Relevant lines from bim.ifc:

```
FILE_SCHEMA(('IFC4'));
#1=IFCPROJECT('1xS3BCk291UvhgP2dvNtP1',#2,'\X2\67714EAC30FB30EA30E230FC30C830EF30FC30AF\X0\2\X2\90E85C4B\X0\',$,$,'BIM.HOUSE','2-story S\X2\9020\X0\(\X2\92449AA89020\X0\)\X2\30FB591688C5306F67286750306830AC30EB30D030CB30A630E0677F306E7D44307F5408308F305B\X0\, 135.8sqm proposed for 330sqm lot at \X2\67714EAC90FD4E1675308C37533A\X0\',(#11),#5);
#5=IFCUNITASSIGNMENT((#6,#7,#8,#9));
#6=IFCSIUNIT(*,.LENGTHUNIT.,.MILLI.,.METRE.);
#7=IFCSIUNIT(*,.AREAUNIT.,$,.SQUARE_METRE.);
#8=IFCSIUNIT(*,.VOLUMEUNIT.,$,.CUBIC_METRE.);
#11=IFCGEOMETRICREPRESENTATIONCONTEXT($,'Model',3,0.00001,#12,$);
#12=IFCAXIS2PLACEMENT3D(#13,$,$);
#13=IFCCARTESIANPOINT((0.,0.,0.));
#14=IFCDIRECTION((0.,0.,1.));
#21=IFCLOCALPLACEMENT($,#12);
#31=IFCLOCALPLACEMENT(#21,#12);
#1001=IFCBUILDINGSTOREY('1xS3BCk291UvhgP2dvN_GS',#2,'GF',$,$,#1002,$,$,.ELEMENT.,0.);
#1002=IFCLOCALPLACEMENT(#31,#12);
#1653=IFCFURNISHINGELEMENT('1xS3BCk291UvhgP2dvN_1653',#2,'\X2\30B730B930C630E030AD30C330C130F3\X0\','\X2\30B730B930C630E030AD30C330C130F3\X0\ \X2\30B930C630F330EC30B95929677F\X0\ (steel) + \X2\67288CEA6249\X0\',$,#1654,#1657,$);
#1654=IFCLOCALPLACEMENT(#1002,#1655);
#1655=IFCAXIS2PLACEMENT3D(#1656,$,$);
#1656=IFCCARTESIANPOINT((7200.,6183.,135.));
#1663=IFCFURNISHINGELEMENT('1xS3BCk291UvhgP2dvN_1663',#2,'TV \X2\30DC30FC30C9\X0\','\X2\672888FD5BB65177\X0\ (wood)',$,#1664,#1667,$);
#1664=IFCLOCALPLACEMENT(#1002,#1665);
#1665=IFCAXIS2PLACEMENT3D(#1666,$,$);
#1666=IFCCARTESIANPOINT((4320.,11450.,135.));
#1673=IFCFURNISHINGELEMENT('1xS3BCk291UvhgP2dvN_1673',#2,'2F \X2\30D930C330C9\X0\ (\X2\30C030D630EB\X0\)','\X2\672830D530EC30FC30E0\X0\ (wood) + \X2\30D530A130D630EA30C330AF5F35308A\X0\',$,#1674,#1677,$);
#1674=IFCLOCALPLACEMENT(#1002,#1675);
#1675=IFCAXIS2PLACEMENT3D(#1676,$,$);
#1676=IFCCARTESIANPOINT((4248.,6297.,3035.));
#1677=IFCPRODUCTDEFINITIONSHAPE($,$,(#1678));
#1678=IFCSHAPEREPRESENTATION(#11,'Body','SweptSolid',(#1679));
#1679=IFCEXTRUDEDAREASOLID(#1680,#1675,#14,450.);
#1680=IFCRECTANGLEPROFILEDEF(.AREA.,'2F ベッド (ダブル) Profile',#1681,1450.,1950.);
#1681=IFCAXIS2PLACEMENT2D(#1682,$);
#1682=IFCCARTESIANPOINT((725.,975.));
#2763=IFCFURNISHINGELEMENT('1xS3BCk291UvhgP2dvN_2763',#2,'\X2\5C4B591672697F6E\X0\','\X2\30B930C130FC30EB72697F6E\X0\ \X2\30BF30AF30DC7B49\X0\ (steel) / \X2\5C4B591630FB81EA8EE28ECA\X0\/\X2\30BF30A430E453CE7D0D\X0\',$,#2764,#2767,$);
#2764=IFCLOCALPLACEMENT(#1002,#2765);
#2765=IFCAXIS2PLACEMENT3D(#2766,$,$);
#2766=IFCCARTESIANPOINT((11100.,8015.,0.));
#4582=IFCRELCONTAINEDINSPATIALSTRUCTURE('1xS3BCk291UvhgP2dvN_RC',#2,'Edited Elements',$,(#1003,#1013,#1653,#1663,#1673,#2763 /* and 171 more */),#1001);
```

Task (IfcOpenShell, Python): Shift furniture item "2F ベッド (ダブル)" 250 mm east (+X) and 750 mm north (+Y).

```python
import ifcopenshell
import ifcopenshell.api.geometry
import ifcopenshell.util.placement
import ifcopenshell.util.unit

model = ifcopenshell.open("bim.ifc")
unit_scale = ifcopenshell.util.unit.calculate_unit_scale(model)

item = model.by_guid("1xS3BCk291UvhgP2dvN_1673")
matrix = ifcopenshell.util.placement.get_local_placement(item.ObjectPlacement)
matrix[0, 3] += 0.25 / unit_scale
matrix[1, 3] += 0.75 / unit_scale
ifcopenshell.api.geometry.edit_object_placement(model, product=item, matrix=matrix, is_si=False)

print(ifcopenshell.util.placement.get_local_placement(item.ObjectPlacement).round(3) + 0.0)

model.write("bim_rev.ifc")
```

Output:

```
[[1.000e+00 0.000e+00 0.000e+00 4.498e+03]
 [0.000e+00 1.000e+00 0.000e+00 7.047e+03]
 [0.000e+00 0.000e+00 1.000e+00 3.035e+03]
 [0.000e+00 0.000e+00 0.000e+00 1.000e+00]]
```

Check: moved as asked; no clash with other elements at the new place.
